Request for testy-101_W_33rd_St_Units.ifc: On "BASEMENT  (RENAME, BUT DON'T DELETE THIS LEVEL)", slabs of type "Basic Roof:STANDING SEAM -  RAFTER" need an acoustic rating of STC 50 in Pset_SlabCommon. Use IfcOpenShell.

First a look at what the model holds.

```python
import ifcopenshell
import ifcopenshell.util.element

model = ifcopenshell.open("testy-101_W_33rd_St_Units.ifc")
print(model.schema)
storey = next(s for s in model.by_type("IfcBuildingStorey") if s.Name == "BASEMENT  (RENAME, BUT DON'T DELETE THIS LEVEL)")
slabs = [e for e in ifcopenshell.util.element.get_decomposition(storey) if e.is_a("IfcSlab")]
seen = {}
for e in slabs:
    element_type = ifcopenshell.util.element.get_type(e)
    key = (element_type.Name if element_type != e and element_type else None, ifcopenshell.util.element.get_pset(e, "Pset_SlabCommon", "AcousticRating"))
    seen[key] = seen.get(key, 0) + 1
for (name, value), count in sorted(seen.items(), key=str):
    print(count, "x", name, "|", value)
```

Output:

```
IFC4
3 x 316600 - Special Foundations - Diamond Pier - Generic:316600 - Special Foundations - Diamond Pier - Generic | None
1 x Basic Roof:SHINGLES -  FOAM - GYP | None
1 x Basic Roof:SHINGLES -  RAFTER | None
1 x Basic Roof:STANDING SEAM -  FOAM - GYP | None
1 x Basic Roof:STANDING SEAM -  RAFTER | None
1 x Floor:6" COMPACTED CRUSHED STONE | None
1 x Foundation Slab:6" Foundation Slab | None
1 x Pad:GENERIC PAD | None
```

```python
import ifcopenshell
import ifcopenshell.api.pset
import ifcopenshell.util.element

model = ifcopenshell.open("testy-101_W_33rd_St_Units.ifc")

storey = next(s for s in model.by_type("IfcBuildingStorey") if s.Name == "BASEMENT  (RENAME, BUT DON'T DELETE THIS LEVEL)")
slabs = [e for e in ifcopenshell.util.element.get_decomposition(storey) if e.is_a("IfcSlab")]

count = 0
for e in slabs:
    element_type = ifcopenshell.util.element.get_type(e)
    if element_type in (None, e) or element_type.Name != "Basic Roof:STANDING SEAM -  RAFTER":
        continue
    # add_pset returns the element's existing set when there is one.
    pset = ifcopenshell.api.pset.add_pset(model, product=e, name="Pset_SlabCommon")
    ifcopenshell.api.pset.edit_pset(model, pset=pset, properties={"AcousticRating": "STC 50"})
    count += 1

print(count, "slabs updated")

model.write("testy-101_W_33rd_St_Units_v2.ifc")
```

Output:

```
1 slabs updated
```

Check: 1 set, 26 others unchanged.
